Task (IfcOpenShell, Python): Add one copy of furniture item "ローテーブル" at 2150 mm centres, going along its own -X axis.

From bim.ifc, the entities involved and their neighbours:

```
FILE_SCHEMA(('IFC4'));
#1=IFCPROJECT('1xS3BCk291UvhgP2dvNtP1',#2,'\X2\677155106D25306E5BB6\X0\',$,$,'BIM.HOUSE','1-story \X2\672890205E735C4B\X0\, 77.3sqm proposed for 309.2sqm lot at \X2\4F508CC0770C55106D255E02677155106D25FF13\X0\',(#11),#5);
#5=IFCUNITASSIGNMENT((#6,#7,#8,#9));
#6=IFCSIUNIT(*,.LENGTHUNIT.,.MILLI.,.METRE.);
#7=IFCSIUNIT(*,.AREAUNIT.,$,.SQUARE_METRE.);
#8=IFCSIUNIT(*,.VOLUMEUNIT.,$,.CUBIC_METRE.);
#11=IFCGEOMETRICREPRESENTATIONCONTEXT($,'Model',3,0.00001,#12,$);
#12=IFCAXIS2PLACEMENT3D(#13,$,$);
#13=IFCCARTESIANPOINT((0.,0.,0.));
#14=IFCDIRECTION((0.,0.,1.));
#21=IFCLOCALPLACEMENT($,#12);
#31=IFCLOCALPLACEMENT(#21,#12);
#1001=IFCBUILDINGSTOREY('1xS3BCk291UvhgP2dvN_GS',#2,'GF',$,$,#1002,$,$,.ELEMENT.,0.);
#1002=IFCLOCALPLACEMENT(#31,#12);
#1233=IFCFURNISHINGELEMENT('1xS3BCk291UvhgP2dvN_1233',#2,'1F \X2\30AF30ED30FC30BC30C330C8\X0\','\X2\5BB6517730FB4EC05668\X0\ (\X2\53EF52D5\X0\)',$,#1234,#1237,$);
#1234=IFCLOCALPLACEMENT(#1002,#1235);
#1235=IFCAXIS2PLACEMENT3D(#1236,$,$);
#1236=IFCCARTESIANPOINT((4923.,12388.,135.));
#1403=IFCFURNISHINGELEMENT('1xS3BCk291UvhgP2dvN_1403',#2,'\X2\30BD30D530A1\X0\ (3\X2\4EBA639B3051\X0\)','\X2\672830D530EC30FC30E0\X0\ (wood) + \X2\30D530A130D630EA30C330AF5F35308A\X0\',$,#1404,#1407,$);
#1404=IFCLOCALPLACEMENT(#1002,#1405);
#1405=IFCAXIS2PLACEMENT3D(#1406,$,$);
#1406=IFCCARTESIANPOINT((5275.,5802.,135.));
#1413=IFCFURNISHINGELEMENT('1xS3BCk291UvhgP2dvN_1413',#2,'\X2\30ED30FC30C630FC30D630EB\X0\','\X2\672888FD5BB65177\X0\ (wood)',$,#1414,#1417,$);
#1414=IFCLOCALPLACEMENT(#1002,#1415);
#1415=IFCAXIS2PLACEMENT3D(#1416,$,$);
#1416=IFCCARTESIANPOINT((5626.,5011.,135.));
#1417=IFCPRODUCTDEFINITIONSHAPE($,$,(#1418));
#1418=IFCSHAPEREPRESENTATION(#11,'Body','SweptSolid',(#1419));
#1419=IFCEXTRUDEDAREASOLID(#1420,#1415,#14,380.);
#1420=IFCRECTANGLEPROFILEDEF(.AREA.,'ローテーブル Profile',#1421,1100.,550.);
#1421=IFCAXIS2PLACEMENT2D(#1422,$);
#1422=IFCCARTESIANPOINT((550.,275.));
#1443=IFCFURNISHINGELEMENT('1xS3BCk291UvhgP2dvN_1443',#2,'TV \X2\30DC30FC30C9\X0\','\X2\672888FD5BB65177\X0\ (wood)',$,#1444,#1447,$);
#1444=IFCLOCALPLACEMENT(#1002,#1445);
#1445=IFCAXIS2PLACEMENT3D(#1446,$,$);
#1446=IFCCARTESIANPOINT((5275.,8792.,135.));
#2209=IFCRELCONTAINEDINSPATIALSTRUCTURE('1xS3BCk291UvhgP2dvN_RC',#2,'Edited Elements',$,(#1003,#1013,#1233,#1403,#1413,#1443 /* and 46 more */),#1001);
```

```python
import ifcopenshell
import ifcopenshell.api.geometry
import ifcopenshell.api.root
import ifcopenshell.util.element
import ifcopenshell.util.placement

model = ifcopenshell.open("bim.ifc")


def reuse_history(source, copy):
    """copy_class also copies each property set's owner history, people and application; keep the originals."""
    for rel in copy.IsDefinedBy:
        if rel.is_a("IfcRelDefinesByProperties") and (history := rel.RelatingPropertyDefinition.OwnerHistory):
            rel.RelatingPropertyDefinition.OwnerHistory = source.OwnerHistory
            ifcopenshell.util.element.remove_deep2(model, history)


source = model.by_id(1413)
base = ifcopenshell.util.placement.get_local_placement(source.ObjectPlacement)
step = -base[:3, 0] * 2150.0

for i in range(1, 2):
    copy = ifcopenshell.api.root.copy_class(model, product=source)
    copy.Representation = ifcopenshell.util.element.copy_deep(
        model, source.Representation, exclude=["IfcGeometricRepresentationContext", "IfcRepresentationMap"]
    )
    reuse_history(source, copy)
    matrix = base.copy()
    matrix[:3, 3] += i * step
    print("added at", matrix[:3, 3].round(3) + 0.0)
    ifcopenshell.api.geometry.edit_object_placement(model, product=copy, matrix=matrix, is_si=False)

model.write("bim_rev.ifc")
```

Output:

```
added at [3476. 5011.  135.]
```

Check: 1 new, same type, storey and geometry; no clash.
